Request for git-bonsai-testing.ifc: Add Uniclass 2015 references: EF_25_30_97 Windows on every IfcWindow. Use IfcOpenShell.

First a look at what the model holds.

```python
import ifcopenshell

model = ifcopenshell.open("git-bonsai-testing.ifc")
print(model.schema)
print("classifications:", [c.Name for c in model.by_type("IfcClassification")])
for ifc_class in ("IfcDoor", "IfcRoof", "IfcStair", "IfcWall", "IfcWindow"):
    print(ifc_class, len(model.by_type(ifc_class)))
```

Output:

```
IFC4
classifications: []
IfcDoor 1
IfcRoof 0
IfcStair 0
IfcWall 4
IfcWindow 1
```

```python
import ifcopenshell
import ifcopenshell.api.classification

model = ifcopenshell.open("git-bonsai-testing.ifc")

system = ifcopenshell.api.classification.add_classification(model, classification="Uniclass 2015")

codes = {
    "IfcWindow": ("EF_25_30_97", "Windows"),
}
for ifc_class, (code, name) in codes.items():
    products = model.by_type(ifc_class)
    ifcopenshell.api.classification.add_reference(
        model, products=products, classification=system, identification=code, name=name
    )
    print(code, len(products))

model.write("git-bonsai-testing_updated.ifc")
```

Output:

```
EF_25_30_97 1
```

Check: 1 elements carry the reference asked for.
